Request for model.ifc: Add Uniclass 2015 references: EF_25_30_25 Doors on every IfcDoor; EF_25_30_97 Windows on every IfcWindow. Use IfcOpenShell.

First a look at what the model holds.

```python
import ifcopenshell

model = ifcopenshell.open("model.ifc")
print(model.schema)
print("classifications:", [c.Name for c in model.by_type("IfcClassification")])
for ifc_class in ("IfcDoor", "IfcRoof", "IfcStair", "IfcWall", "IfcWindow"):
    print(ifc_class, len(model.by_type(ifc_class)))
```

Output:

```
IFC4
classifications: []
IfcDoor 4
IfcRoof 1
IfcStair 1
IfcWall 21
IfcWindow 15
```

```python
import ifcopenshell
import ifcopenshell.api.classification

model = ifcopenshell.open("model.ifc")

system = ifcopenshell.api.classification.add_classification(model, classification="Uniclass 2015")

codes = {
    "IfcDoor": ("EF_25_30_25", "Doors"),
    "IfcWindow": ("EF_25_30_97", "Windows"),
}
for ifc_class, (code, name) in codes.items():
    products = model.by_type(ifc_class)
    ifcopenshell.api.classification.add_reference(
        model, products=products, classification=system, identification=code, name=name
    )
    print(code, len(products))

model.write("model_updated.ifc")
```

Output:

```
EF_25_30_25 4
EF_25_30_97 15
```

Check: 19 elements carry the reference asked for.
